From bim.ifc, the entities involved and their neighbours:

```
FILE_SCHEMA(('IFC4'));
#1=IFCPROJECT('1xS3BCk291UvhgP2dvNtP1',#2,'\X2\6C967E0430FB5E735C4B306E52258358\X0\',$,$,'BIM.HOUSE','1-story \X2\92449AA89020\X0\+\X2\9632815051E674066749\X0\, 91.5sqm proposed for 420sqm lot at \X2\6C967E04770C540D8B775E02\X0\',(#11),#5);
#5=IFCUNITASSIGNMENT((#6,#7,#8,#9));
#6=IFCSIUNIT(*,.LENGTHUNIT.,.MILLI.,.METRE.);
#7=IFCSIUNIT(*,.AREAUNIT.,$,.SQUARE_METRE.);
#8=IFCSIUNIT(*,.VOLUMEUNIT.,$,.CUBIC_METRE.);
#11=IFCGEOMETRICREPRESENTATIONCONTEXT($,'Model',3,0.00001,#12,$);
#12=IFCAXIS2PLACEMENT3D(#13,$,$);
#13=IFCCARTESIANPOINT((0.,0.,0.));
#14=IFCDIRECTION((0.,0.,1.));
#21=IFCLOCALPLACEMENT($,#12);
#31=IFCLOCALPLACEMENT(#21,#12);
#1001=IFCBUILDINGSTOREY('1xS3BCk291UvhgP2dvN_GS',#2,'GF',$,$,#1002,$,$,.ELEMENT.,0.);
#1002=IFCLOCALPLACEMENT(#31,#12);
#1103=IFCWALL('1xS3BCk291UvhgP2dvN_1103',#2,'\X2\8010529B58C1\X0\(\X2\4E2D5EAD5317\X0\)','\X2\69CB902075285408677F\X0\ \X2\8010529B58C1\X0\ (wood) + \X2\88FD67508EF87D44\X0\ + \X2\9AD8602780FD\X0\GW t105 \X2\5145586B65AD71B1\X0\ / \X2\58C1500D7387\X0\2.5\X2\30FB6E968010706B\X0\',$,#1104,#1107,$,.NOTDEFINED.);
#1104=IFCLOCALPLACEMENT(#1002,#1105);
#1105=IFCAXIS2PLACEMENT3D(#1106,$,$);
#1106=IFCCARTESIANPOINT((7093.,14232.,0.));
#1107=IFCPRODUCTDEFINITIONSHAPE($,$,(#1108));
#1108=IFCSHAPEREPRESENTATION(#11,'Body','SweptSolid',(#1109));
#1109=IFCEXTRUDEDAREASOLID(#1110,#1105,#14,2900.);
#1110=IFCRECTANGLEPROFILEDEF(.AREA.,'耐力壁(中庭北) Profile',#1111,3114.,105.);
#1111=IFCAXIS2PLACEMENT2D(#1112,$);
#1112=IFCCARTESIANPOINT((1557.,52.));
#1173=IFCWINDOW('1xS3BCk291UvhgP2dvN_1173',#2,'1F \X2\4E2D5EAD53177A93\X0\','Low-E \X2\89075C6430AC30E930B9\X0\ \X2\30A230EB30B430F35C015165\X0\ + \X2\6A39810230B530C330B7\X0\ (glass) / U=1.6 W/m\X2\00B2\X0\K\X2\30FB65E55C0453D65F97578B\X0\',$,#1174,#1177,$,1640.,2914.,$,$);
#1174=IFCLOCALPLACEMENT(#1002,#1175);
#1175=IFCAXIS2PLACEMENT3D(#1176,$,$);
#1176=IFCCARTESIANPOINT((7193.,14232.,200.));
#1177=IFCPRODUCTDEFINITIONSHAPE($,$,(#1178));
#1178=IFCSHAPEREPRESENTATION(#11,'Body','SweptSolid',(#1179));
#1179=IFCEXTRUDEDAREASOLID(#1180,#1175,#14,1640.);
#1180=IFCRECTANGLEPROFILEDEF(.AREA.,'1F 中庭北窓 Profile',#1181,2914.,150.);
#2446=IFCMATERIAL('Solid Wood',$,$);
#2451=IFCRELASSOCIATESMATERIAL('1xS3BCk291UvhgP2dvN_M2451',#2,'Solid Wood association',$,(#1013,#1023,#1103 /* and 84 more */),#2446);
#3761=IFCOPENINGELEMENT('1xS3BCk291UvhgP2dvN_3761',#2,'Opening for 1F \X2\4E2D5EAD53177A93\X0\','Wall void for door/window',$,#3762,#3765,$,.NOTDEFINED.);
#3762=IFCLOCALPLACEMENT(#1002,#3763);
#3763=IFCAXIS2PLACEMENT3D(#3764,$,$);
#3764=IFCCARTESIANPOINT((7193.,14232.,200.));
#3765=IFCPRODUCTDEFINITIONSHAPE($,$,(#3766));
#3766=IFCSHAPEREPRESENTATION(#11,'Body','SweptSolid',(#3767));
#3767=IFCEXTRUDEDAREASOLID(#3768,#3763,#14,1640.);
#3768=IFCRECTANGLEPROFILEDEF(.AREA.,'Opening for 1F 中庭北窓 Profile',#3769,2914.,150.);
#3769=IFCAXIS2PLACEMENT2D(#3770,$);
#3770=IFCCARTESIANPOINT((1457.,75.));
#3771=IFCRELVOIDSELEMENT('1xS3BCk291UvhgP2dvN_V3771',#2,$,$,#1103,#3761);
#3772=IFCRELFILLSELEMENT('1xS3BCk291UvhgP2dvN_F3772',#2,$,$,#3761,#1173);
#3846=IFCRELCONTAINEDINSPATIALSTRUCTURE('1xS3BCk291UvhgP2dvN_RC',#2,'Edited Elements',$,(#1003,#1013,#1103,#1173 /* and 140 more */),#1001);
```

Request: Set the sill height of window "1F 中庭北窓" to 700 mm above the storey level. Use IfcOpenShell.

```python
import numpy as np
import ifcopenshell
import ifcopenshell.api.geometry
import ifcopenshell.geom
import ifcopenshell.util.element
import ifcopenshell.util.placement
import ifcopenshell.util.shape
import ifcopenshell.util.unit

model = ifcopenshell.open("bim.ifc")
unit_scale = ifcopenshell.util.unit.calculate_unit_scale(model)

window = model.by_id(1173)
opening = window.FillsVoids[0].RelatingOpeningElement
storey = ifcopenshell.util.element.get_container(window, ifc_class="IfcBuildingStorey")
level = ifcopenshell.util.placement.get_local_placement(storey.ObjectPlacement)[2, 3]

# The opening's origin need not be at the sill, so measure its lowest point.
shape = ifcopenshell.geom.create_shape(ifcopenshell.geom.settings(), opening)
bottom = ifcopenshell.util.shape.get_shape_bottom_elevation(shape, shape.geometry) / unit_scale
dz = level + 0.7 / unit_scale - bottom

shift = np.array([0.0, 0.0, dz])
# The window is not placed relative to its opening, so move both.
for product in (opening, window):
    matrix = ifcopenshell.util.placement.get_local_placement(product.ObjectPlacement)
    matrix[:3, 3] += shift
    ifcopenshell.api.geometry.edit_object_placement(model, product=product, matrix=matrix, is_si=False)

print(f"moved by {dz * unit_scale:+.3f} m")

model.write("bim_rev.ifc")
```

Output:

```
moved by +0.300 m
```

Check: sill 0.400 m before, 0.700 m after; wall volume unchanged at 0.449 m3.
